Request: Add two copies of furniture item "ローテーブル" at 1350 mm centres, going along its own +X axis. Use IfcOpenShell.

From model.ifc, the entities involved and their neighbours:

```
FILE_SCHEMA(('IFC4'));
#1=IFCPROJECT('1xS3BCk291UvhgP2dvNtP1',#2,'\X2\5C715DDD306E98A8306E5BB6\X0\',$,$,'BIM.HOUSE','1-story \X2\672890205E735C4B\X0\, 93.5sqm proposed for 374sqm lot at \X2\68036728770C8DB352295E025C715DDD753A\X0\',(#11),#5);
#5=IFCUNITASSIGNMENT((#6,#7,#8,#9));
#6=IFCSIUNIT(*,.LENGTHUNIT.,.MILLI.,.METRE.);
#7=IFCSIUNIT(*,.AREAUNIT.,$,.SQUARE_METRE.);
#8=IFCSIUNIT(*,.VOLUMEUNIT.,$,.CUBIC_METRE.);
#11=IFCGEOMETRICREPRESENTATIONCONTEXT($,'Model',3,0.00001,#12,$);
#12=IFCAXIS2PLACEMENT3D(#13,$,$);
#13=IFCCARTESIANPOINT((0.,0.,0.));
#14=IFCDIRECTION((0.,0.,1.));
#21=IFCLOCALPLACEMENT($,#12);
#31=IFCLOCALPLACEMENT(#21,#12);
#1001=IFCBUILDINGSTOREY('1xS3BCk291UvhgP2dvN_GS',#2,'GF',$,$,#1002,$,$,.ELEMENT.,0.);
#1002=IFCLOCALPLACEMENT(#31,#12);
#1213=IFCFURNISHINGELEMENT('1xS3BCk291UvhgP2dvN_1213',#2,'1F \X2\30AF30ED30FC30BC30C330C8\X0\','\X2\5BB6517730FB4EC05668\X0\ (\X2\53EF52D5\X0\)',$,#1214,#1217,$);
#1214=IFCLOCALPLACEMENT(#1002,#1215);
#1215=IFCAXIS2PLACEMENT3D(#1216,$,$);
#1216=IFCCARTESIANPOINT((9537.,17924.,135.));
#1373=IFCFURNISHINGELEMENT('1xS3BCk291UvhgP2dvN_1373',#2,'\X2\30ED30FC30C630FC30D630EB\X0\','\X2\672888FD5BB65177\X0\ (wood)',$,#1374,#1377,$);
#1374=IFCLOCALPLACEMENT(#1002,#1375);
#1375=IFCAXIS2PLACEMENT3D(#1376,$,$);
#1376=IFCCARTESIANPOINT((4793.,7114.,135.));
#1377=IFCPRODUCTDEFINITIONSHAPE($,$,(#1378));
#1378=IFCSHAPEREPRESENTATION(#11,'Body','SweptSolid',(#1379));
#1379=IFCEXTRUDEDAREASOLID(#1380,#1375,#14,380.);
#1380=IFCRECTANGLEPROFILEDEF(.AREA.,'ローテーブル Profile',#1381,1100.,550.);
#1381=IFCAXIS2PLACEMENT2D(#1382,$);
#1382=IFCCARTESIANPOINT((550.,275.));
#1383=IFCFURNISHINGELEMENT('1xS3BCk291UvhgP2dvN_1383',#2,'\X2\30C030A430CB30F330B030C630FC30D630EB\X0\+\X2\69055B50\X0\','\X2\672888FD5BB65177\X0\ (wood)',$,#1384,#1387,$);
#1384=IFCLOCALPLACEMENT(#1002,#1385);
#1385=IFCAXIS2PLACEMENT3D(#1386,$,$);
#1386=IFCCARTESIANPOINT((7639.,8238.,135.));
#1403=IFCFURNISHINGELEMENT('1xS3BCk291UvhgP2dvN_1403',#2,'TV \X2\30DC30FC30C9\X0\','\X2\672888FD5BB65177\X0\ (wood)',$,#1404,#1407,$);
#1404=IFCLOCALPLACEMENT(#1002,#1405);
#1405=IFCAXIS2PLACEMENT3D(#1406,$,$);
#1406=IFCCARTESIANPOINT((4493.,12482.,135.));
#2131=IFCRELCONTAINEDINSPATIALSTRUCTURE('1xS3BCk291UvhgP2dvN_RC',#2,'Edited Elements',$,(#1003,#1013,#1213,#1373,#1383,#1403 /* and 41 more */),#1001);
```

```python
import ifcopenshell
import ifcopenshell.api.geometry
import ifcopenshell.api.root
import ifcopenshell.util.element
import ifcopenshell.util.placement
import ifcopenshell.util.unit

model = ifcopenshell.open("model.ifc")
unit_scale = ifcopenshell.util.unit.calculate_unit_scale(model)


def reuse_history(source, copy):
    """copy_class also copies each property set's owner history, people and application; keep the originals."""
    for rel in copy.IsDefinedBy:
        if rel.is_a("IfcRelDefinesByProperties") and (history := rel.RelatingPropertyDefinition.OwnerHistory):
            rel.RelatingPropertyDefinition.OwnerHistory = source.OwnerHistory
            ifcopenshell.util.element.remove_deep2(model, history)


source = model.by_guid("1xS3BCk291UvhgP2dvN_1373")
base = ifcopenshell.util.placement.get_local_placement(source.ObjectPlacement)
step = base[:3, 0] * 1.35 / unit_scale

for i in range(1, 3):
    copy = ifcopenshell.api.root.copy_class(model, product=source)
    copy.Representation = ifcopenshell.util.element.copy_deep(
        model, source.Representation, exclude=["IfcGeometricRepresentationContext", "IfcRepresentationMap"]
    )
    reuse_history(source, copy)
    matrix = base.copy()
    matrix[:3, 3] += i * step
    print("added at", matrix[:3, 3].round(3) + 0.0)
    ifcopenshell.api.geometry.edit_object_placement(model, product=copy, matrix=matrix, is_si=False)

model.write("model_rev.ifc")
```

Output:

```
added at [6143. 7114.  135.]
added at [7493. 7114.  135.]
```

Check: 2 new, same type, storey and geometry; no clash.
